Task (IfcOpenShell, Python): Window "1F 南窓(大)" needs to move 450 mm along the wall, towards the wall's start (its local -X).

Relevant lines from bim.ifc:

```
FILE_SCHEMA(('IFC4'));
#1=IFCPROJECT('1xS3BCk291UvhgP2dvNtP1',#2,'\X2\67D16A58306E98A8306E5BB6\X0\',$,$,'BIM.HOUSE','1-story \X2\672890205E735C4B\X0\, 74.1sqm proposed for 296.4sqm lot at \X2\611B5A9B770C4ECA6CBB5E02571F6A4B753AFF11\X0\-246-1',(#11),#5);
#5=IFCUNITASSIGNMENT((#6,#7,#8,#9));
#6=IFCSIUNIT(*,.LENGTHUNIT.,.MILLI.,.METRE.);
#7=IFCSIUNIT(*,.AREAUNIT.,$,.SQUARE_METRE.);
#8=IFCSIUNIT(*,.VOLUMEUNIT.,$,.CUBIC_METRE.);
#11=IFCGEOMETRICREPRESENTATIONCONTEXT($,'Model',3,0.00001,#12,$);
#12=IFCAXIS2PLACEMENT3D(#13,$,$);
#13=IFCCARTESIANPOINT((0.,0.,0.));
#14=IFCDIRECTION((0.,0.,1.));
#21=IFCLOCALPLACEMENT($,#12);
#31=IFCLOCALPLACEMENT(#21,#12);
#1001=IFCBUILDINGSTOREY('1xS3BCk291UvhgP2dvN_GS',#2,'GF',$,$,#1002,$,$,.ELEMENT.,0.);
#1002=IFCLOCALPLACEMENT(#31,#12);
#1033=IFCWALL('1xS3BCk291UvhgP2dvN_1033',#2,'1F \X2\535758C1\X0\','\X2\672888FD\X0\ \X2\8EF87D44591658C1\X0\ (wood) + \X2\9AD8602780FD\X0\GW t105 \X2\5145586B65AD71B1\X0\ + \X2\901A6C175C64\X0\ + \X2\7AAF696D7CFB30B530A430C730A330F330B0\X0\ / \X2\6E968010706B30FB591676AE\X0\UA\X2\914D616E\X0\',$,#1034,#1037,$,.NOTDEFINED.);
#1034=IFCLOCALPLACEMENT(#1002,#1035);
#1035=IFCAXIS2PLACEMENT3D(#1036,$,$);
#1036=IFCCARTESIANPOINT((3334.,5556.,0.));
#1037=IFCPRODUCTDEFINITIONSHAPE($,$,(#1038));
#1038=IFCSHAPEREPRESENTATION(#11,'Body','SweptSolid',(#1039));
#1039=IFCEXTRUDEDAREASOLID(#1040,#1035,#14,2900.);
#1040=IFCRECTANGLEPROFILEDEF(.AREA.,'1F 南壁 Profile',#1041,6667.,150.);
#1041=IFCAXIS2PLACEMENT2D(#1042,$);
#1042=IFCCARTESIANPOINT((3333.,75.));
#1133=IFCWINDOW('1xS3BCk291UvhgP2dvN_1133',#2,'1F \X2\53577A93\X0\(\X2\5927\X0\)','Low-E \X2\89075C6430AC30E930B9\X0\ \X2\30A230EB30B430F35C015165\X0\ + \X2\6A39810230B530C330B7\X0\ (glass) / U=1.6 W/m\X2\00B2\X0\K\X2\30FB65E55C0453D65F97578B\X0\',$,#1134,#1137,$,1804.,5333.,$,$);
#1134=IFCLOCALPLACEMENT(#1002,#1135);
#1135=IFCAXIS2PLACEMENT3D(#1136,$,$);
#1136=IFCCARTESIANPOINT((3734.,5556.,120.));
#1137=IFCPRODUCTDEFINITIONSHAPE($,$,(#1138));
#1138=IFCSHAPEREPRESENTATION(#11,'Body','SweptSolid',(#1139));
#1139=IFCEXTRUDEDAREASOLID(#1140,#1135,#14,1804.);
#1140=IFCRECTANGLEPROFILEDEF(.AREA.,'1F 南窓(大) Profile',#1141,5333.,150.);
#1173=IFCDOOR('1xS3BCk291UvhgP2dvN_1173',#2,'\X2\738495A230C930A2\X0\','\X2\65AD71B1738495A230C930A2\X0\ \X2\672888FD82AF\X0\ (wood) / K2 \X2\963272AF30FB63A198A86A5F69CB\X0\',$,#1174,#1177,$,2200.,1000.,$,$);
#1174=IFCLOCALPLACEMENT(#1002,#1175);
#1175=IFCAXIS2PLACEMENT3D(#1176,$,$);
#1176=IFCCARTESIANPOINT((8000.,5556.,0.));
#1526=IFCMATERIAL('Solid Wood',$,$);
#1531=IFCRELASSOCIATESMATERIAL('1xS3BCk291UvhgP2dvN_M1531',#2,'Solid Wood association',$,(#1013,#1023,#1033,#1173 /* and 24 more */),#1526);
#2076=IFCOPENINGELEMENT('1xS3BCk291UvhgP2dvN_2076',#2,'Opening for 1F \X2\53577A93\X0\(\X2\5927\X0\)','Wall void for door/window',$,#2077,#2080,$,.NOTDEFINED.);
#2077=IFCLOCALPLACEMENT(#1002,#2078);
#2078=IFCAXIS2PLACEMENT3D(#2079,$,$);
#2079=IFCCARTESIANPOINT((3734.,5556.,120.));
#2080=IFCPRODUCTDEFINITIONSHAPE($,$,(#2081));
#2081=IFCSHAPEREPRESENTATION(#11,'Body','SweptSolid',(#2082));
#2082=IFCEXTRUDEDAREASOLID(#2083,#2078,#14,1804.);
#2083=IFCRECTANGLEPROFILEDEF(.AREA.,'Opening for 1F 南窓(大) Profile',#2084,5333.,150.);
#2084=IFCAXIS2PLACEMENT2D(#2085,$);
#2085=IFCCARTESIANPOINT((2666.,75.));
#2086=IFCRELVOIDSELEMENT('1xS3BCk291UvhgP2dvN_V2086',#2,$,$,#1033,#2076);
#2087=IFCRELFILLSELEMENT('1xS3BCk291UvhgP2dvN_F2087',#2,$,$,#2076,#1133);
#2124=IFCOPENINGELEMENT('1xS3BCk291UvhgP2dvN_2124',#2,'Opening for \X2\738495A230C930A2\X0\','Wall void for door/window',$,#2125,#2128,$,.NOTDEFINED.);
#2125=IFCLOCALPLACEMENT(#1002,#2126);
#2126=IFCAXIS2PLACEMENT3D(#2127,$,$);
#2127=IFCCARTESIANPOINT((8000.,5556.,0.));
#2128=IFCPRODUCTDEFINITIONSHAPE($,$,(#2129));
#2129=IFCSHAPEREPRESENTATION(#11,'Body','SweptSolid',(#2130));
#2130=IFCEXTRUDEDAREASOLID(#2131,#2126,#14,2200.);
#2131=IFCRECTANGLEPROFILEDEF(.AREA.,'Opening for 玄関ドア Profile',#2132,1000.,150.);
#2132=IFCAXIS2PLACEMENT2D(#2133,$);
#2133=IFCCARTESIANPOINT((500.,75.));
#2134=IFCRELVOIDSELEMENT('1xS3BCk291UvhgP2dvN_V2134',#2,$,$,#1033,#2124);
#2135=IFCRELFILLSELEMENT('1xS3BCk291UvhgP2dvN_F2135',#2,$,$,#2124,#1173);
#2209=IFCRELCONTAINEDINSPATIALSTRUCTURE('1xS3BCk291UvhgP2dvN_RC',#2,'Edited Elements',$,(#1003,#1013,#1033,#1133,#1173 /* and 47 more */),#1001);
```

```python
import ifcopenshell
import ifcopenshell.api.geometry
import ifcopenshell.util.placement

model = ifcopenshell.open("bim.ifc")

window = model.by_guid("1xS3BCk291UvhgP2dvN_1133")
opening = window.FillsVoids[0].RelatingOpeningElement
wall = opening.VoidsElements[0].RelatingBuildingElement

wall_matrix = ifcopenshell.util.placement.get_local_placement(wall.ObjectPlacement)
shift = wall_matrix[:3, 0] * -450.0
before = ifcopenshell.util.placement.get_local_placement(window.ObjectPlacement)[:3, 3].copy()

# The window is not placed relative to its opening, so move both.
for product in (opening, window):
    matrix = ifcopenshell.util.placement.get_local_placement(product.ObjectPlacement)
    matrix[:3, 3] += shift
    ifcopenshell.api.geometry.edit_object_placement(model, product=product, matrix=matrix, is_si=False)

after = ifcopenshell.util.placement.get_local_placement(window.ObjectPlacement)[:3, 3]
print("window moved by", (after - before).round(3) + 0.0)

model.write("bim_updated.ifc")
```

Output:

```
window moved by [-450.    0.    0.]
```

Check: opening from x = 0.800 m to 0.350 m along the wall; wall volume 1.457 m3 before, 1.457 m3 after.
